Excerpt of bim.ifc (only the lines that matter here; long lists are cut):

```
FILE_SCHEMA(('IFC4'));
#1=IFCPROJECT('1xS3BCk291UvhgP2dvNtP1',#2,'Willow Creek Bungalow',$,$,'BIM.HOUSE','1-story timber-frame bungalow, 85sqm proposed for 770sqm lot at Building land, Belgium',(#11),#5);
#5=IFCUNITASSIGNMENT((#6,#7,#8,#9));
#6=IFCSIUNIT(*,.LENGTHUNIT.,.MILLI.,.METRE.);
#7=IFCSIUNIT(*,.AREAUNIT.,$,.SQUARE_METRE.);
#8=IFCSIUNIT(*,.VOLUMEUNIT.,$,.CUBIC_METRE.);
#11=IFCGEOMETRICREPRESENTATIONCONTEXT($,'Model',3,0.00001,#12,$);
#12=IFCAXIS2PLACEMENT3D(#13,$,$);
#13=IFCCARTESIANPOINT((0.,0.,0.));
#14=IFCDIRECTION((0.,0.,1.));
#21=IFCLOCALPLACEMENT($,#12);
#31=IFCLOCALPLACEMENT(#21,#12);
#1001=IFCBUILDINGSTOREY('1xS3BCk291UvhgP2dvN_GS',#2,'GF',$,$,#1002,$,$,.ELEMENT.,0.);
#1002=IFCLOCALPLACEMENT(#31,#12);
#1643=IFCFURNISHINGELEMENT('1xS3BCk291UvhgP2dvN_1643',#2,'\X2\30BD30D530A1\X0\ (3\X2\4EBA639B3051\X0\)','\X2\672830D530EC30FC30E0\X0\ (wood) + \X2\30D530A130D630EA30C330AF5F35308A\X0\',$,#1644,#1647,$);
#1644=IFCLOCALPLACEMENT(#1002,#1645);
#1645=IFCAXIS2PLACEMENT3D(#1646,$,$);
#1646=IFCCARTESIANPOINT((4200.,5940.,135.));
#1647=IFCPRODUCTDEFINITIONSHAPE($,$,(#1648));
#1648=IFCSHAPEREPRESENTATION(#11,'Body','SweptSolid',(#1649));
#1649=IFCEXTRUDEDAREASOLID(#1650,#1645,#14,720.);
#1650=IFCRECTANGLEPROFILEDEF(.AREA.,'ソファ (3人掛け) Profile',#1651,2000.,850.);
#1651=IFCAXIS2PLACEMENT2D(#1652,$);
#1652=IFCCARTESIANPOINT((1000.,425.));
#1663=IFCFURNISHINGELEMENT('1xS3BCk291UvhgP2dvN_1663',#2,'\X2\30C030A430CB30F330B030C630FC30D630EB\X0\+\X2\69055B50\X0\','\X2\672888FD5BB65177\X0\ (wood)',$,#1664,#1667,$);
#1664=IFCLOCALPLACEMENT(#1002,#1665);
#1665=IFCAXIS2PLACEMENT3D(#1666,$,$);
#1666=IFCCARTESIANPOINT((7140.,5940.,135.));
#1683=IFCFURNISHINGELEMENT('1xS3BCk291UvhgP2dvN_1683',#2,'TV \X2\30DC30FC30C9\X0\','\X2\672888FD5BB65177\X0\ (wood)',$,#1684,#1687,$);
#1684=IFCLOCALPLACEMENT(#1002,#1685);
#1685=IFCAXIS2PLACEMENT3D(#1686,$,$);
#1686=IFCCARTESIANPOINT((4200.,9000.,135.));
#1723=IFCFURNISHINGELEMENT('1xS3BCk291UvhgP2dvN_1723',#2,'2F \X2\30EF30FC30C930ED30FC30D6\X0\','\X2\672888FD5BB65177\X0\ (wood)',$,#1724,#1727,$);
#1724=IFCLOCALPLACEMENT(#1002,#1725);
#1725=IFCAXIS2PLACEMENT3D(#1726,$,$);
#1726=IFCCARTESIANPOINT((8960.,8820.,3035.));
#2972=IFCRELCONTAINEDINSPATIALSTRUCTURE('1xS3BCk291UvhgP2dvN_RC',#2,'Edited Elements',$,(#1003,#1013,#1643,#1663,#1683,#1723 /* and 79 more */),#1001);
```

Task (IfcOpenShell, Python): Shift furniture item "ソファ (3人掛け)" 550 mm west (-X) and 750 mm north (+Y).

```python
import ifcopenshell
import ifcopenshell.api.geometry
import ifcopenshell.util.placement

model = ifcopenshell.open("bim.ifc")

item = model.by_id(1643)
matrix = ifcopenshell.util.placement.get_local_placement(item.ObjectPlacement)
matrix[0, 3] -= 550.0
matrix[1, 3] += 750.0
ifcopenshell.api.geometry.edit_object_placement(model, product=item, matrix=matrix, is_si=False)

print(ifcopenshell.util.placement.get_local_placement(item.ObjectPlacement).round(3) + 0.0)

model.write("bim_updated.ifc")
```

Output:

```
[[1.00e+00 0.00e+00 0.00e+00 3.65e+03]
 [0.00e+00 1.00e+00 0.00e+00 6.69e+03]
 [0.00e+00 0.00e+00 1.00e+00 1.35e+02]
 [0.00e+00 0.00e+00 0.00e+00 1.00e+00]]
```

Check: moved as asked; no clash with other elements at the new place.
